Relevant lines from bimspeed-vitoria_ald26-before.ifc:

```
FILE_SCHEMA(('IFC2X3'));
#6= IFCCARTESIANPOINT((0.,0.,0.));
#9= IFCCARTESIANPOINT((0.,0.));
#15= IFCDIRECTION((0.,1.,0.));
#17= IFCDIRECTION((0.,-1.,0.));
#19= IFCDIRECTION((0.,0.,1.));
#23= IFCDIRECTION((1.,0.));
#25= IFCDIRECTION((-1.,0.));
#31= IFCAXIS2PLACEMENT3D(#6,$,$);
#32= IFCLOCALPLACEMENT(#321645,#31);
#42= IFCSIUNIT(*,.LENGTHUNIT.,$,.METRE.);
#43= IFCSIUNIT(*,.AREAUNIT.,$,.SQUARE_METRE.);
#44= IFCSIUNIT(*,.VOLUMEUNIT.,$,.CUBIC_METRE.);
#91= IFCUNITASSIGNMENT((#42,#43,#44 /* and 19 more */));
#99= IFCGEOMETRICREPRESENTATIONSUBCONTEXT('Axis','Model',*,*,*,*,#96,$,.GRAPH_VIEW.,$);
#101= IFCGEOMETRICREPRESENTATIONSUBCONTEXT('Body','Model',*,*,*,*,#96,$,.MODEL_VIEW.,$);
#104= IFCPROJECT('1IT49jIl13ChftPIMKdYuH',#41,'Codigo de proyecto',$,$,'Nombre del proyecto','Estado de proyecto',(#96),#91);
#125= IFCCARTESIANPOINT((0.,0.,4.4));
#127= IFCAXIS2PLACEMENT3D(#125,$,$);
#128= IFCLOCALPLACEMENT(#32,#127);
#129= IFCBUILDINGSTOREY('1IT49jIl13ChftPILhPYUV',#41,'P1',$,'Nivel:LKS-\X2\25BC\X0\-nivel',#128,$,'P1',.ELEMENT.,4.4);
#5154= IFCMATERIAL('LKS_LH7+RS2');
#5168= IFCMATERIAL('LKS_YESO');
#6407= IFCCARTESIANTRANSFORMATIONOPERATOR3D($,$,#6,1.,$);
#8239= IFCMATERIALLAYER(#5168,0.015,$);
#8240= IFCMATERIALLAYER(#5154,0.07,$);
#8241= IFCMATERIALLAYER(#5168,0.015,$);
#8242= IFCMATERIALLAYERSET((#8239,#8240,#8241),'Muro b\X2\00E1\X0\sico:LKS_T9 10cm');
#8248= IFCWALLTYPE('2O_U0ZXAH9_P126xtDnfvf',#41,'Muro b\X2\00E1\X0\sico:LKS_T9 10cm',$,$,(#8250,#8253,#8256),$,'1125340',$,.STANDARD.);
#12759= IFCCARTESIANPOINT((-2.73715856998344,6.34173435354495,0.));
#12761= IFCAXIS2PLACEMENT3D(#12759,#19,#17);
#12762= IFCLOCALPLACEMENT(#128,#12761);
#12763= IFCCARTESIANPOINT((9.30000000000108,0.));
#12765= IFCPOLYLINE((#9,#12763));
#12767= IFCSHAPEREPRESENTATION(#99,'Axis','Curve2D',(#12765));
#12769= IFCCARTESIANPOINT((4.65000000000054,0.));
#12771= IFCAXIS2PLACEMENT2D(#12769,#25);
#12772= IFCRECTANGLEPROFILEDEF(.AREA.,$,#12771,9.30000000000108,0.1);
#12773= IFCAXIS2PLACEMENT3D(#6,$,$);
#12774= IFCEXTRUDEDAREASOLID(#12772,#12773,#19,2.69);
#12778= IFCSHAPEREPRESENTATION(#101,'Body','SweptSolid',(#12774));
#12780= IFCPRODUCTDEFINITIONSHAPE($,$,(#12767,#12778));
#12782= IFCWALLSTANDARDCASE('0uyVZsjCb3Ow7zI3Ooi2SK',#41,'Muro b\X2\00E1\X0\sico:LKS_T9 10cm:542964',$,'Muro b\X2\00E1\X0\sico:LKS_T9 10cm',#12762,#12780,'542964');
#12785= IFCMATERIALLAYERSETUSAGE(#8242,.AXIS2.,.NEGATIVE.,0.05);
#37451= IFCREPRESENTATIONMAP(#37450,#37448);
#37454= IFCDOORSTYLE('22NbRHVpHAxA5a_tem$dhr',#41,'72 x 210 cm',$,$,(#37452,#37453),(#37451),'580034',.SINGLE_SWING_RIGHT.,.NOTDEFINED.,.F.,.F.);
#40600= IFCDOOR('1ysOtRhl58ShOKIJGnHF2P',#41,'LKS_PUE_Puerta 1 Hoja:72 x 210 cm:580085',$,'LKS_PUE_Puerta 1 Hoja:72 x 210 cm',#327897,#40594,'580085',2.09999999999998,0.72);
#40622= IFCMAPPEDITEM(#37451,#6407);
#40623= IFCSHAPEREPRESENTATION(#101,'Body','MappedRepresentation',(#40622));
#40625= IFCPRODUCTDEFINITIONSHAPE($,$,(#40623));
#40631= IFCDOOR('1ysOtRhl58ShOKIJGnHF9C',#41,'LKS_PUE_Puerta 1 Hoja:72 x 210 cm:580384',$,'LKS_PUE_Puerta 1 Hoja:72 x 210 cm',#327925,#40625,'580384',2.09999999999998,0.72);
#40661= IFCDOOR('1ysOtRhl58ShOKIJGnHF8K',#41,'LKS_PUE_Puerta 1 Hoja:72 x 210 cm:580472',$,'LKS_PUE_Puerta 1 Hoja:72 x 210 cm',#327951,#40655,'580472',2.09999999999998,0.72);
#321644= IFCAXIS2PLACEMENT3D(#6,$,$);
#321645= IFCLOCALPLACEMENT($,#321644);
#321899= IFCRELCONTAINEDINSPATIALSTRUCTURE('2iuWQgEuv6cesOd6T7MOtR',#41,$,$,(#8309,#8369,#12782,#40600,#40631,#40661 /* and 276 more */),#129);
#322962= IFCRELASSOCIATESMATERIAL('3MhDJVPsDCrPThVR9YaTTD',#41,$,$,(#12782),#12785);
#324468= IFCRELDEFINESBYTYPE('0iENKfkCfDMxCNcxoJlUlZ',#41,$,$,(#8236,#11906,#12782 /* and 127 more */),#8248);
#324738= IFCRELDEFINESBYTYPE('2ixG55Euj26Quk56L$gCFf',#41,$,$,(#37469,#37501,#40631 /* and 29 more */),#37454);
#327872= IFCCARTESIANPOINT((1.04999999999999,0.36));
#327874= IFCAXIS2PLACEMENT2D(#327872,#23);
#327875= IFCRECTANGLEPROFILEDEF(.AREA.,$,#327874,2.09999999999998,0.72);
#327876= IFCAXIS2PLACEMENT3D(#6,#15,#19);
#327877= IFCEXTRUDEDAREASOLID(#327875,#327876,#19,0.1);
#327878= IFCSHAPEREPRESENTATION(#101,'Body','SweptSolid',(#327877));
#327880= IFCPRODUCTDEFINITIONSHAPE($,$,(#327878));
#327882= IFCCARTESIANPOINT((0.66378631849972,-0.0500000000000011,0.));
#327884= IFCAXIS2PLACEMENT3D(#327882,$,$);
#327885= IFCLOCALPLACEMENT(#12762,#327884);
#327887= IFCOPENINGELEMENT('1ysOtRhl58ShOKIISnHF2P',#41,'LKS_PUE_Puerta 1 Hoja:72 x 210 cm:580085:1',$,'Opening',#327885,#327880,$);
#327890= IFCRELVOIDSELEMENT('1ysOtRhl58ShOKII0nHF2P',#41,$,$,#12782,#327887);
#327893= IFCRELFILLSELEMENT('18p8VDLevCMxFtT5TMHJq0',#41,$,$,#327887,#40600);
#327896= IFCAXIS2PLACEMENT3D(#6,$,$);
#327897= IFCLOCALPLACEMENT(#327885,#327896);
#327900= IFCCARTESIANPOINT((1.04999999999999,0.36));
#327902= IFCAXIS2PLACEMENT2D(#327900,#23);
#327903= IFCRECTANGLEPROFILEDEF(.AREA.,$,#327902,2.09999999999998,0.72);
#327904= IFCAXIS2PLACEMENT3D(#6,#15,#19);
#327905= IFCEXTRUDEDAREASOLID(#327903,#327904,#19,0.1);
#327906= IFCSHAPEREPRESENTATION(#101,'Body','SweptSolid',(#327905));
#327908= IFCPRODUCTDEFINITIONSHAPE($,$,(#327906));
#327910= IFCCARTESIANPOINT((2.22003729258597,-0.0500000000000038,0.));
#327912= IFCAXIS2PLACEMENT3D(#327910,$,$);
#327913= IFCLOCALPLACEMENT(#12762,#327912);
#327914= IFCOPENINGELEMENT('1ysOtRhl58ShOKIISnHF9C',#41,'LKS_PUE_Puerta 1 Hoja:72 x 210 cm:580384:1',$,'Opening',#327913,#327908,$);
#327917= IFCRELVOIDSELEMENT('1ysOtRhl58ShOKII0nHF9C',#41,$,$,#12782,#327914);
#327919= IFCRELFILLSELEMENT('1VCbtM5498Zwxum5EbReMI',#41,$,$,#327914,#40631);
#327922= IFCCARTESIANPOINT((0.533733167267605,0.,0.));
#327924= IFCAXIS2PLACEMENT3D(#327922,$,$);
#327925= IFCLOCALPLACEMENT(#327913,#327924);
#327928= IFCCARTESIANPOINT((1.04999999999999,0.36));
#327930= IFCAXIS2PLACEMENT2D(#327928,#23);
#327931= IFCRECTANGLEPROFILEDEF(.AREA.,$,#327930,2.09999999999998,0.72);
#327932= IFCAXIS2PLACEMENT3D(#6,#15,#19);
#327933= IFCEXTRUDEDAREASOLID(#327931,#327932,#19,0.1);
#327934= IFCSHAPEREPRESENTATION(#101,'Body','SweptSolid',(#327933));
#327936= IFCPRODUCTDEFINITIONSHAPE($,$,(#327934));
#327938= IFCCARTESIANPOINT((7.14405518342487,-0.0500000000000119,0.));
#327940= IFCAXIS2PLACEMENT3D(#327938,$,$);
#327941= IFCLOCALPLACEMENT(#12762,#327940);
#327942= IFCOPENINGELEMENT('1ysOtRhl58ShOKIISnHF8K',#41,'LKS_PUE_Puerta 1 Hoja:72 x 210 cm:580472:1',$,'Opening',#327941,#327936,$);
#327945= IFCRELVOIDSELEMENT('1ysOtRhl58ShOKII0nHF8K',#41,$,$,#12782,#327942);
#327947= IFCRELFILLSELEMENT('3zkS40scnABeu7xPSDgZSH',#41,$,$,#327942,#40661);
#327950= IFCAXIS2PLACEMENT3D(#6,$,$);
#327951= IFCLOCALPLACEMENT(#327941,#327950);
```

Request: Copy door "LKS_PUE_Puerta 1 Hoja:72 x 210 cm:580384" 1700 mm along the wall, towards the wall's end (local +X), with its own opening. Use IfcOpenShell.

```python
import ifcopenshell
import ifcopenshell.api.feature
import ifcopenshell.api.geometry
import ifcopenshell.api.root
import ifcopenshell.geom
import ifcopenshell.util.element
import ifcopenshell.util.placement
import ifcopenshell.util.shape
import ifcopenshell.util.unit

model = ifcopenshell.open("bimspeed-vitoria_ald26-before.ifc")
unit_scale = ifcopenshell.util.unit.calculate_unit_scale(model)
settings = ifcopenshell.geom.settings()


def volume(element):
    """Net volume in cubic metres, openings subtracted."""
    shape = ifcopenshell.geom.create_shape(settings, element)
    return ifcopenshell.util.shape.get_volume(shape.geometry)


def reuse_history(source, copy):
    """copy_class also copies each property set's owner history, people and application; keep the originals."""
    for rel in copy.IsDefinedBy:
        if rel.is_a("IfcRelDefinesByProperties") and (history := rel.RelatingPropertyDefinition.OwnerHistory):
            rel.RelatingPropertyDefinition.OwnerHistory = source.OwnerHistory
            ifcopenshell.util.element.remove_deep2(model, history)


door = model.by_guid("1ysOtRhl58ShOKIJGnHF9C")
opening = door.FillsVoids[0].RelatingOpeningElement
wall = opening.VoidsElements[0].RelatingBuildingElement
before = volume(wall)
shift = ifcopenshell.util.placement.get_local_placement(wall.ObjectPlacement)[:3, 0] * 1.7 / unit_scale

# copy_class copies the void relationship, type, container and properties, but no geometry.
new_opening = ifcopenshell.api.root.copy_class(model, product=opening)
new_opening.Representation = ifcopenshell.util.element.copy_deep(
    model, opening.Representation, exclude=["IfcGeometricRepresentationContext", "IfcRepresentationMap"]
)
new_opening.Name = "LKS_PUE_Puerta 1 Hoja:72 x 210 cm"
new_door = ifcopenshell.api.root.copy_class(model, product=door)
new_door.Representation = ifcopenshell.util.element.copy_deep(
    model, door.Representation, exclude=["IfcGeometricRepresentationContext", "IfcRepresentationMap"]
)
new_door.Name = "LKS_PUE_Puerta 1 Hoja:72 x 210 cm"
new_door.Tag = None
reuse_history(door, new_door)
fills = ifcopenshell.api.feature.add_filling(model, opening=new_opening, element=new_door)
fills.OwnerHistory = new_door.OwnerHistory  # required in IFC2X3

for old, new in ((opening, new_opening), (door, new_door)):
    matrix = ifcopenshell.util.placement.get_local_placement(old.ObjectPlacement)
    matrix[:3, 3] += shift
    ifcopenshell.api.geometry.edit_object_placement(model, product=new, matrix=matrix, is_si=False)

after = volume(wall)

print(f"wall volume {before:.3f} -> {after:.3f} m3")

model.write("bimspeed-vitoria_ald26-before_edited.ifc")
```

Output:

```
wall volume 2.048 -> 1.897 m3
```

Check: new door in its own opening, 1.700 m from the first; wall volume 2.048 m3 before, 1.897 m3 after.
